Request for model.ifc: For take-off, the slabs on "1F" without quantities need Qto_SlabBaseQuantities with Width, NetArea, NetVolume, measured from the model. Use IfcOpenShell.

First a look at what the model holds.

```python
import ifcopenshell
import ifcopenshell.util.element
import ifcopenshell.util.unit

model = ifcopenshell.open("model.ifc")
print(model.schema)
for unit_type in ("LENGTHUNIT", "AREAUNIT", "VOLUMEUNIT"):
    print(unit_type, ifcopenshell.util.unit.calculate_unit_scale(model, unit_type))
storey = next(s for s in model.by_type("IfcBuildingStorey") if s.Name == "1F")
slabs = [e for e in ifcopenshell.util.element.get_decomposition(storey) if e.is_a("IfcSlab")]
for e in sorted(slabs, key=lambda e: e.id()):
    print(e.id(), e.is_a(), e.Name, list(ifcopenshell.util.element.get_psets(e, qtos_only=True)), sep=" | ")
```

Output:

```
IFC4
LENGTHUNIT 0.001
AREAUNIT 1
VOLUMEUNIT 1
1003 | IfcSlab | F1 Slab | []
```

```python
import ifcopenshell
import ifcopenshell.api.pset
import ifcopenshell.geom
import ifcopenshell.util.element
import ifcopenshell.util.shape
import ifcopenshell.util.unit

model = ifcopenshell.open("model.ifc")
unit_scale = ifcopenshell.util.unit.calculate_unit_scale(model)
area_scale = ifcopenshell.util.unit.calculate_unit_scale(model, "AREAUNIT")
volume_scale = ifcopenshell.util.unit.calculate_unit_scale(model, "VOLUMEUNIT")
settings = ifcopenshell.geom.settings()

storey = next(s for s in model.by_type("IfcBuildingStorey") if s.Name == "1F")
slabs = [e for e in ifcopenshell.util.element.get_decomposition(storey) if e.is_a("IfcSlab")]

for e in sorted(slabs, key=lambda e: e.id()):
    if ifcopenshell.util.element.get_psets(e, qtos_only=True, should_inherit=False):
        continue
    # Geometry comes back in metres, in the element's own axes.
    shape = ifcopenshell.geom.create_shape(settings, e)
    values = {
        "Width": ifcopenshell.util.shape.get_z(shape.geometry) / unit_scale,
        "NetArea": ifcopenshell.util.shape.get_footprint_area(shape.geometry) / area_scale,
        "NetVolume": ifcopenshell.util.shape.get_volume(shape.geometry) / volume_scale,
    }
    qto = ifcopenshell.api.pset.add_qto(model, product=e, name="Qto_SlabBaseQuantities")
    ifcopenshell.api.pset.edit_qto(model, qto=qto, properties=values)
    print(e.id(), {k: round(v, 3) for k, v in values.items()})

model.write("model_updated.ifc")
```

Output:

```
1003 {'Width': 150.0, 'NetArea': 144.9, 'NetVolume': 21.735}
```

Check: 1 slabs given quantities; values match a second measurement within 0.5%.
